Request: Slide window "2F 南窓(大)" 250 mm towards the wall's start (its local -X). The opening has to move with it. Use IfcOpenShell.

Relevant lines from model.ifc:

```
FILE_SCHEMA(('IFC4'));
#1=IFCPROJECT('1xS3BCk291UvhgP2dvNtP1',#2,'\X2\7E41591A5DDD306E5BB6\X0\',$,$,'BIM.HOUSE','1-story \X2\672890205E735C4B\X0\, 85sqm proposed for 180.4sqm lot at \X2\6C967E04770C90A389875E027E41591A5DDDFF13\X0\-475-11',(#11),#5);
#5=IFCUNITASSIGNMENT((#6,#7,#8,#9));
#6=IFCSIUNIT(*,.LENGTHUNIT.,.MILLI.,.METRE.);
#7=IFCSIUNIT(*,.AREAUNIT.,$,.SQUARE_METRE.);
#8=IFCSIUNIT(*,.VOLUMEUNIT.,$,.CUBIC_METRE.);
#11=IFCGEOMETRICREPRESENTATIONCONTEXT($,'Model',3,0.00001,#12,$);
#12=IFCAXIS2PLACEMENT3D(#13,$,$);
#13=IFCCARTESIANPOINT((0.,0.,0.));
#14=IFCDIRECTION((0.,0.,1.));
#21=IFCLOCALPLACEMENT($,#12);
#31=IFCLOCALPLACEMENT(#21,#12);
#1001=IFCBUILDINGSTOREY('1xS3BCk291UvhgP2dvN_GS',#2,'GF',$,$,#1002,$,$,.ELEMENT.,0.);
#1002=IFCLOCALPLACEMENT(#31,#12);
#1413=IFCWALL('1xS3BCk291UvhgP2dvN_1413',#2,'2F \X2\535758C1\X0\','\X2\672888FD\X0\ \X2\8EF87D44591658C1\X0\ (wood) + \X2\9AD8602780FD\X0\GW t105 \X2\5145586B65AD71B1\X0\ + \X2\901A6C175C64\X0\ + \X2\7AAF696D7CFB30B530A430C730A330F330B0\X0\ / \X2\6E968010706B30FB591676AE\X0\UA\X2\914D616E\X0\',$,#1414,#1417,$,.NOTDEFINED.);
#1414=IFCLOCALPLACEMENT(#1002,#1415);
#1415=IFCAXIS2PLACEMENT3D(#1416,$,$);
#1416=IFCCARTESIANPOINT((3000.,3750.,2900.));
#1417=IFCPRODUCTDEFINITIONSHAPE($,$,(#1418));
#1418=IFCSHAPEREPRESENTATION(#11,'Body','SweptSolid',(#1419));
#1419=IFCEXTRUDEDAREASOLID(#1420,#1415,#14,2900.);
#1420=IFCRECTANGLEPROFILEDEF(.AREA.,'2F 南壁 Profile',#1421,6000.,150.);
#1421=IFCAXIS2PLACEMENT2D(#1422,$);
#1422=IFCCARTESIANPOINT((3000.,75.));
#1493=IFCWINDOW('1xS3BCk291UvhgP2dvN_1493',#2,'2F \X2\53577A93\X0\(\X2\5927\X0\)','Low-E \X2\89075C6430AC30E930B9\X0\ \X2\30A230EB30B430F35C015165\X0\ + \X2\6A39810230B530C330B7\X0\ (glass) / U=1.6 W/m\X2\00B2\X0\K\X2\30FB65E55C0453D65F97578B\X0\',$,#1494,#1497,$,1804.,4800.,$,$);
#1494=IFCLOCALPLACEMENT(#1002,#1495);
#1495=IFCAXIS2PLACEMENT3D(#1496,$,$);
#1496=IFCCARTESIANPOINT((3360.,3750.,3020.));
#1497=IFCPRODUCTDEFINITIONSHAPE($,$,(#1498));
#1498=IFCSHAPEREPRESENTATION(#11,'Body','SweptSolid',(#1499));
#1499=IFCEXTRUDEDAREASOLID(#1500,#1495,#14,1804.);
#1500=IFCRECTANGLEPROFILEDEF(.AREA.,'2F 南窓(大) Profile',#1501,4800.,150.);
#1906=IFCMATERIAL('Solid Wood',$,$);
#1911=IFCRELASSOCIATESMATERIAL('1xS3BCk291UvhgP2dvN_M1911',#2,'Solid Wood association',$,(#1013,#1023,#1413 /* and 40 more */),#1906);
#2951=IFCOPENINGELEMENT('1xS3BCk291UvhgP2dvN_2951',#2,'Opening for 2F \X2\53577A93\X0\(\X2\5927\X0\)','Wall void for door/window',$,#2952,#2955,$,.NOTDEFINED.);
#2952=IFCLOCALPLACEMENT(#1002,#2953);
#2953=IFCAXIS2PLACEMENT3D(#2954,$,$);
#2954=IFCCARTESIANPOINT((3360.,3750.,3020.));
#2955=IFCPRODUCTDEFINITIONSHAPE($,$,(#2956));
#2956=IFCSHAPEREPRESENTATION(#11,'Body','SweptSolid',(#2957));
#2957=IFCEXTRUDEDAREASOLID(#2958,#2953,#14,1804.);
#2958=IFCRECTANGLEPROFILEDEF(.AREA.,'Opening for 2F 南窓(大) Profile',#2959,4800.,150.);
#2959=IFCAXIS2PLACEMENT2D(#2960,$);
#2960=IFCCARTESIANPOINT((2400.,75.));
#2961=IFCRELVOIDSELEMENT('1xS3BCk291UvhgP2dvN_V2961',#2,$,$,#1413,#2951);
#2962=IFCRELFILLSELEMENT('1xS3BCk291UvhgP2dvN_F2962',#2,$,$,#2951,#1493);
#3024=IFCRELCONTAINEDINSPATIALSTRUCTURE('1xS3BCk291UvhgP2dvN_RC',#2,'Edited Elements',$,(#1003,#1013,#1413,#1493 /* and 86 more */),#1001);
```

```python
import ifcopenshell
import ifcopenshell.api.geometry
import ifcopenshell.util.placement

model = ifcopenshell.open("model.ifc")

window = model.by_guid("1xS3BCk291UvhgP2dvN_1493")
opening = window.FillsVoids[0].RelatingOpeningElement
wall = opening.VoidsElements[0].RelatingBuildingElement

wall_matrix = ifcopenshell.util.placement.get_local_placement(wall.ObjectPlacement)
shift = wall_matrix[:3, 0] * -250.0
before = ifcopenshell.util.placement.get_local_placement(window.ObjectPlacement)[:3, 3].copy()

# The window is not placed relative to its opening, so move both.
for product in (opening, window):
    matrix = ifcopenshell.util.placement.get_local_placement(product.ObjectPlacement)
    matrix[:3, 3] += shift
    ifcopenshell.api.geometry.edit_object_placement(model, product=product, matrix=matrix, is_si=False)

after = ifcopenshell.util.placement.get_local_placement(window.ObjectPlacement)[:3, 3]
print("window moved by", (after - before).round(3) + 0.0)

model.write("model_v2.ifc")
```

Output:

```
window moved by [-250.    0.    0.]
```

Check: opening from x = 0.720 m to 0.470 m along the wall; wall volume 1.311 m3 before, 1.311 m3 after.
